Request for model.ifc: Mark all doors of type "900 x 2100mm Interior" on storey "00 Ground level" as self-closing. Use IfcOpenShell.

First a look at what the model holds.

```python
import ifcopenshell
import ifcopenshell.util.element

model = ifcopenshell.open("model.ifc")
print(model.schema)
storey = next(s for s in model.by_type("IfcBuildingStorey") if s.Name == "00 Ground level")
doors = [e for e in ifcopenshell.util.element.get_decomposition(storey) if e.is_a("IfcDoor")]
seen = {}
for e in doors:
    element_type = ifcopenshell.util.element.get_type(e)
    key = (element_type.Name if element_type != e and element_type else None, ifcopenshell.util.element.get_pset(e, "Pset_DoorCommon", "SelfClosing"))
    seen[key] = seen.get(key, 0) + 1
for (name, value), count in sorted(seen.items(), key=str):
    print(count, "x", name, "|", value)
```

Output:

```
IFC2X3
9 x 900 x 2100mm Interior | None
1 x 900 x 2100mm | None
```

```python
import ifcopenshell
import ifcopenshell.api.pset
import ifcopenshell.util.element

model = ifcopenshell.open("model.ifc")

storey = next(s for s in model.by_type("IfcBuildingStorey") if s.Name == "00 Ground level")
doors = [e for e in ifcopenshell.util.element.get_decomposition(storey) if e.is_a("IfcDoor")]

count = 0
for e in doors:
    element_type = ifcopenshell.util.element.get_type(e)
    if element_type in (None, e) or element_type.Name != "900 x 2100mm Interior":
        continue
    # add_pset returns the element's existing set when there is one.
    pset = ifcopenshell.api.pset.add_pset(model, product=e, name="Pset_DoorCommon")
    ifcopenshell.api.pset.edit_pset(model, pset=pset, properties={"SelfClosing": True})
    count += 1

print(count, "doors updated")

model.write("model_rev.ifc")
```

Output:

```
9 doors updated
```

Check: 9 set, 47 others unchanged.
